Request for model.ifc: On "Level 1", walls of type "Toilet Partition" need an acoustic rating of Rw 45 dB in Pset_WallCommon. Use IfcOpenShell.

First a look at what the model holds.

```python
import ifcopenshell
import ifcopenshell.util.element

model = ifcopenshell.open("model.ifc")
print(model.schema)
storey = next(s for s in model.by_type("IfcBuildingStorey") if s.Name == "Level 1")
walls = [e for e in ifcopenshell.util.element.get_decomposition(storey) if e.is_a("IfcWall")]
seen = {}
for e in walls:
    element_type = ifcopenshell.util.element.get_type(e)
    key = (element_type.Name if element_type != e and element_type else None, ifcopenshell.util.element.get_pset(e, "Pset_WallCommon", "AcousticRating"))
    seen[key] = seen.get(key, 0) + 1
for (name, value), count in sorted(seen.items(), key=str):
    print(count, "x", name, "|", value)
```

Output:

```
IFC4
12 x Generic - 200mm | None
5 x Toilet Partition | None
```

```python
import ifcopenshell
import ifcopenshell.api.pset
import ifcopenshell.util.element

model = ifcopenshell.open("model.ifc")

storey = next(s for s in model.by_type("IfcBuildingStorey") if s.Name == "Level 1")
walls = [e for e in ifcopenshell.util.element.get_decomposition(storey) if e.is_a("IfcWall")]

count = 0
for e in walls:
    element_type = ifcopenshell.util.element.get_type(e)
    if element_type in (None, e) or element_type.Name != "Toilet Partition":
        continue
    # add_pset returns the element's existing set when there is one.
    pset = ifcopenshell.api.pset.add_pset(model, product=e, name="Pset_WallCommon")
    ifcopenshell.api.pset.edit_pset(model, pset=pset, properties={"AcousticRating": "Rw 45 dB"})
    count += 1

print(count, "walls updated")

model.write("model_updated.ifc")
```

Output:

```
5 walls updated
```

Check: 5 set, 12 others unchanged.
